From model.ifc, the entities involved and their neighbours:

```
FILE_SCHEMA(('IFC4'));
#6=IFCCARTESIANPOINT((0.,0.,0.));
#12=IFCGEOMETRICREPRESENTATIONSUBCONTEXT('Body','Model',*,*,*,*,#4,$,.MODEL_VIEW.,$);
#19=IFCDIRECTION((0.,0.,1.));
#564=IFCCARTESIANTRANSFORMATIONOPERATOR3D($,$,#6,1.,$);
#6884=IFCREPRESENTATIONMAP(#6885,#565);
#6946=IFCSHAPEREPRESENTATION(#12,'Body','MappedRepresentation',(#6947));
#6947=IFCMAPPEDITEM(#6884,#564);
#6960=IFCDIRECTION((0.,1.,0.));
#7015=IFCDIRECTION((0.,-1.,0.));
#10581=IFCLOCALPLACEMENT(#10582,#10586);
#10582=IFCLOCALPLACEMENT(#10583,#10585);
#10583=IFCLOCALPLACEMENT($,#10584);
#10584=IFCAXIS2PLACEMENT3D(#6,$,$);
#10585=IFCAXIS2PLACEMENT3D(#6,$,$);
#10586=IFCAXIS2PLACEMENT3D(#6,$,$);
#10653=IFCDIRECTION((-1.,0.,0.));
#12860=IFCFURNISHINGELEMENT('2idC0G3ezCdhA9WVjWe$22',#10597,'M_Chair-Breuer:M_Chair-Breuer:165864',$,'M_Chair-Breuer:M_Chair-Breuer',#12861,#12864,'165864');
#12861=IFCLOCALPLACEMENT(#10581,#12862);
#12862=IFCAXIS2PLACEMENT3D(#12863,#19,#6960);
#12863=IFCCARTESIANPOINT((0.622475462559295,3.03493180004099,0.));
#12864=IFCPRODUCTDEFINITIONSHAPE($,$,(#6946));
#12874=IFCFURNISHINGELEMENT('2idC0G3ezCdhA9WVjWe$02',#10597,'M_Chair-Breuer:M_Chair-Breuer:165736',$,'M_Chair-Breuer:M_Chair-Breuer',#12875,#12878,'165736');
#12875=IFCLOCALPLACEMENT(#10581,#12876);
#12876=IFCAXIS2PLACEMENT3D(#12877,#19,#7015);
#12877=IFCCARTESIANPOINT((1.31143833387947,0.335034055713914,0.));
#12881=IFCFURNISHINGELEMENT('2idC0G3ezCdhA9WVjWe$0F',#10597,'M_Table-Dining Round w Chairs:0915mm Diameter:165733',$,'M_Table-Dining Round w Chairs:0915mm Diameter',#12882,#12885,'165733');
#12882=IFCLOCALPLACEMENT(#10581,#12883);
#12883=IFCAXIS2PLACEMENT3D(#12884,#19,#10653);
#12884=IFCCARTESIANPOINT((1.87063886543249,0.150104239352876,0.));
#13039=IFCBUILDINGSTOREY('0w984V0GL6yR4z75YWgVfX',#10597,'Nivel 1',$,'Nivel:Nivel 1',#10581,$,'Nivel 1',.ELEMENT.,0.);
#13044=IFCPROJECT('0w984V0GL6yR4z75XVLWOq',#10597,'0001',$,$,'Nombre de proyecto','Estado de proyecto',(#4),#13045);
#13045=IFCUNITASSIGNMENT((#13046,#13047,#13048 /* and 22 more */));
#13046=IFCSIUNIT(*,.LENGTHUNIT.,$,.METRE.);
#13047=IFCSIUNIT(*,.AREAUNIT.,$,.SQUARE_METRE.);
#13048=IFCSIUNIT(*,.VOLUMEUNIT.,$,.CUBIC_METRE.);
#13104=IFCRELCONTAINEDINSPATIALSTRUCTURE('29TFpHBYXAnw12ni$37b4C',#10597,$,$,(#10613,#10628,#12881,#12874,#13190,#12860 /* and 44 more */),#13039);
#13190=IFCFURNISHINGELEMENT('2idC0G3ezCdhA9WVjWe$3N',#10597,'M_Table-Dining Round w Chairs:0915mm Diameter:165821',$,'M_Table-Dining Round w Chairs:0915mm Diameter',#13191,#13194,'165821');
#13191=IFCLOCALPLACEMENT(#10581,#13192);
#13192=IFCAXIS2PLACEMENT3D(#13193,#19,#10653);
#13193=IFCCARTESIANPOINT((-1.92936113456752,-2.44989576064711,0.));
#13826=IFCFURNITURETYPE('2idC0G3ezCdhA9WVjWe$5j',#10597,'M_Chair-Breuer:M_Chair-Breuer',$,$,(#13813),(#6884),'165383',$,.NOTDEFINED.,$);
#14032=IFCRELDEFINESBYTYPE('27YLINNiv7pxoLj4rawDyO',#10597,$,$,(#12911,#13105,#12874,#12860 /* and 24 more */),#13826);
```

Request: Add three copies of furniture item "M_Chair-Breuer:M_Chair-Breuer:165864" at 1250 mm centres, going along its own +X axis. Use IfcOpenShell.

```python
import ifcopenshell
import ifcopenshell.api.geometry
import ifcopenshell.api.root
import ifcopenshell.util.element
import ifcopenshell.util.placement
import ifcopenshell.util.unit

model = ifcopenshell.open("model.ifc")
unit_scale = ifcopenshell.util.unit.calculate_unit_scale(model)


def reuse_history(source, copy):
    """copy_class also copies each property set's owner history, people and application; keep the originals."""
    for rel in copy.IsDefinedBy:
        if rel.is_a("IfcRelDefinesByProperties") and (history := rel.RelatingPropertyDefinition.OwnerHistory):
            rel.RelatingPropertyDefinition.OwnerHistory = source.OwnerHistory
            ifcopenshell.util.element.remove_deep2(model, history)


source = model.by_id(12860)
base = ifcopenshell.util.placement.get_local_placement(source.ObjectPlacement)
step = base[:3, 0] * 1.25 / unit_scale

for i in range(1, 4):
    copy = ifcopenshell.api.root.copy_class(model, product=source)
    copy.Representation = ifcopenshell.util.element.copy_deep(
        model, source.Representation, exclude=["IfcGeometricRepresentationContext", "IfcRepresentationMap"]
    )
    copy.Name = "M_Chair-Breuer:M_Chair-Breuer"
    copy.Tag = None
    reuse_history(source, copy)
    matrix = base.copy()
    matrix[:3, 3] += i * step
    print("added at", matrix[:3, 3].round(3) + 0.0)
    ifcopenshell.api.geometry.edit_object_placement(model, product=copy, matrix=matrix, is_si=False)

model.write("model_edited.ifc")
```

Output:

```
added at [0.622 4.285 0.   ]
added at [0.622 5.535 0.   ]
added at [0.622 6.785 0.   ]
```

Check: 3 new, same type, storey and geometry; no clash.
